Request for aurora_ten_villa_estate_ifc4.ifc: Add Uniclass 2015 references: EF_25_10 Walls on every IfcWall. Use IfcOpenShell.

First a look at what the model holds.

```python
import ifcopenshell

model = ifcopenshell.open("aurora_ten_villa_estate_ifc4.ifc")
print(model.schema)
print("classifications:", [c.Name for c in model.by_type("IfcClassification")])
for ifc_class in ("IfcDoor", "IfcRoof", "IfcStair", "IfcWall", "IfcWindow"):
    print(ifc_class, len(model.by_type(ifc_class)))
```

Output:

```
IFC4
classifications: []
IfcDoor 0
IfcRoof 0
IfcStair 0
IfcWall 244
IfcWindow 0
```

```python
import ifcopenshell
import ifcopenshell.api.classification

model = ifcopenshell.open("aurora_ten_villa_estate_ifc4.ifc")

system = ifcopenshell.api.classification.add_classification(model, classification="Uniclass 2015")

codes = {
    "IfcWall": ("EF_25_10", "Walls"),
}
for ifc_class, (code, name) in codes.items():
    products = model.by_type(ifc_class)
    ifcopenshell.api.classification.add_reference(
        model, products=products, classification=system, identification=code, name=name
    )
    print(code, len(products))

model.write("aurora_ten_villa_estate_ifc4_edited.ifc")
```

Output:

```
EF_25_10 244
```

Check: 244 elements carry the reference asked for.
